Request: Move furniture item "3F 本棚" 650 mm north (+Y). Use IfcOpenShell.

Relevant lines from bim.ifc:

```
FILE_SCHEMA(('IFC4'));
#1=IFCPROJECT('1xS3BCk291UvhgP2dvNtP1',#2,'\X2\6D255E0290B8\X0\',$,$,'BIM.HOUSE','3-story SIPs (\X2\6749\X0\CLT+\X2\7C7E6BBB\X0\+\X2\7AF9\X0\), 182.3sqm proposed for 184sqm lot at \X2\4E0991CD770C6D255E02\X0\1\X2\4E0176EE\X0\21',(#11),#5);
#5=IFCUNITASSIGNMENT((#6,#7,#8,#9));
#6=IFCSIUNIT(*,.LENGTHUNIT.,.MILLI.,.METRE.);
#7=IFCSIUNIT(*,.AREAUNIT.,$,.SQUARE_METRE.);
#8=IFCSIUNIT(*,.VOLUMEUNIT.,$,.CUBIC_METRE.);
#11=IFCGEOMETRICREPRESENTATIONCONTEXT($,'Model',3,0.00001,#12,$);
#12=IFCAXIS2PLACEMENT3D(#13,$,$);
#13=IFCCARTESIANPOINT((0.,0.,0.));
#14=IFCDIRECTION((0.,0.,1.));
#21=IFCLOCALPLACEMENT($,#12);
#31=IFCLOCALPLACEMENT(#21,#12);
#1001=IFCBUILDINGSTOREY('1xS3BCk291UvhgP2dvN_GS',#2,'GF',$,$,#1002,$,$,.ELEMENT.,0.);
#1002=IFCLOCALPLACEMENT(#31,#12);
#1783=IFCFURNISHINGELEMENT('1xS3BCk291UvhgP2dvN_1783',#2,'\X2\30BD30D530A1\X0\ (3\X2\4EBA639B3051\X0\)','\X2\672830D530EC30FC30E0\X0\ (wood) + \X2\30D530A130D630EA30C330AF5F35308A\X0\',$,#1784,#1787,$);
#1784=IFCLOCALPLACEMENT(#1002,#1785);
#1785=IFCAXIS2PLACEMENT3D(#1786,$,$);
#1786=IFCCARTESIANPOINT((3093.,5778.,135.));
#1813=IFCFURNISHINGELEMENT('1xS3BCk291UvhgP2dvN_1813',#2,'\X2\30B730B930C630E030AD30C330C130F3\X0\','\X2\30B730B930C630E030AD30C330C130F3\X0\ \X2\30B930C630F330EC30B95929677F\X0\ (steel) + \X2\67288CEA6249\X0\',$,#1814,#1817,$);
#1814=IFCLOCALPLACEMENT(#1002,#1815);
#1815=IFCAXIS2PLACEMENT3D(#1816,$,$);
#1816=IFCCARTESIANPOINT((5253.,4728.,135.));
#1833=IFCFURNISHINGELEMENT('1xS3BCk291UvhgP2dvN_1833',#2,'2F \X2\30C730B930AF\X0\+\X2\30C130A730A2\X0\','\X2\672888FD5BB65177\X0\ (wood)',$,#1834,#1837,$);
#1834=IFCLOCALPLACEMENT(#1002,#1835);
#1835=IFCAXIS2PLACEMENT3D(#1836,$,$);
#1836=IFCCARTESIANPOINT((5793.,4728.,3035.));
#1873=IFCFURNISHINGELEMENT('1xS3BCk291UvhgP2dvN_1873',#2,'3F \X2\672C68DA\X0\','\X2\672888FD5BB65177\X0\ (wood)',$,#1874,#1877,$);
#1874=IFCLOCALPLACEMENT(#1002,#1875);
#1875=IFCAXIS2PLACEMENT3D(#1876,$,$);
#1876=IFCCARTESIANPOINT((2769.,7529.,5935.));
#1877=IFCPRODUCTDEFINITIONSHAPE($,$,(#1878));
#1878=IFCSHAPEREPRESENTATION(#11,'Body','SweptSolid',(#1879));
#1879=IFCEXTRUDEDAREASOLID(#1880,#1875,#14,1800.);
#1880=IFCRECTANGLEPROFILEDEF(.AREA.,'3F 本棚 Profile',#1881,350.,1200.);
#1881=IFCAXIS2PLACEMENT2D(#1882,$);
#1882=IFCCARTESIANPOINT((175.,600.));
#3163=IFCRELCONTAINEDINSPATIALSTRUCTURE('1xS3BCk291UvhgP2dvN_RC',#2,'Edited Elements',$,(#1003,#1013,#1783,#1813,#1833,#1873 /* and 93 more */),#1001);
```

```python
import ifcopenshell
import ifcopenshell.api.geometry
import ifcopenshell.util.placement
import ifcopenshell.util.unit

model = ifcopenshell.open("bim.ifc")
unit_scale = ifcopenshell.util.unit.calculate_unit_scale(model)

item = model.by_guid("1xS3BCk291UvhgP2dvN_1873")
matrix = ifcopenshell.util.placement.get_local_placement(item.ObjectPlacement)
matrix[1, 3] += 0.65 / unit_scale
ifcopenshell.api.geometry.edit_object_placement(model, product=item, matrix=matrix, is_si=False)

print(ifcopenshell.util.placement.get_local_placement(item.ObjectPlacement).round(3) + 0.0)

model.write("bim_edited.ifc")
```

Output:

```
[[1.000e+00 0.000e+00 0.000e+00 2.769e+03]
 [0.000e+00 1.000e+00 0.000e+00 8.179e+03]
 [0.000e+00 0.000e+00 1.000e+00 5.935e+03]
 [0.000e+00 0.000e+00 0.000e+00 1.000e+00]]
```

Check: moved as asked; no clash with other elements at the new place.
